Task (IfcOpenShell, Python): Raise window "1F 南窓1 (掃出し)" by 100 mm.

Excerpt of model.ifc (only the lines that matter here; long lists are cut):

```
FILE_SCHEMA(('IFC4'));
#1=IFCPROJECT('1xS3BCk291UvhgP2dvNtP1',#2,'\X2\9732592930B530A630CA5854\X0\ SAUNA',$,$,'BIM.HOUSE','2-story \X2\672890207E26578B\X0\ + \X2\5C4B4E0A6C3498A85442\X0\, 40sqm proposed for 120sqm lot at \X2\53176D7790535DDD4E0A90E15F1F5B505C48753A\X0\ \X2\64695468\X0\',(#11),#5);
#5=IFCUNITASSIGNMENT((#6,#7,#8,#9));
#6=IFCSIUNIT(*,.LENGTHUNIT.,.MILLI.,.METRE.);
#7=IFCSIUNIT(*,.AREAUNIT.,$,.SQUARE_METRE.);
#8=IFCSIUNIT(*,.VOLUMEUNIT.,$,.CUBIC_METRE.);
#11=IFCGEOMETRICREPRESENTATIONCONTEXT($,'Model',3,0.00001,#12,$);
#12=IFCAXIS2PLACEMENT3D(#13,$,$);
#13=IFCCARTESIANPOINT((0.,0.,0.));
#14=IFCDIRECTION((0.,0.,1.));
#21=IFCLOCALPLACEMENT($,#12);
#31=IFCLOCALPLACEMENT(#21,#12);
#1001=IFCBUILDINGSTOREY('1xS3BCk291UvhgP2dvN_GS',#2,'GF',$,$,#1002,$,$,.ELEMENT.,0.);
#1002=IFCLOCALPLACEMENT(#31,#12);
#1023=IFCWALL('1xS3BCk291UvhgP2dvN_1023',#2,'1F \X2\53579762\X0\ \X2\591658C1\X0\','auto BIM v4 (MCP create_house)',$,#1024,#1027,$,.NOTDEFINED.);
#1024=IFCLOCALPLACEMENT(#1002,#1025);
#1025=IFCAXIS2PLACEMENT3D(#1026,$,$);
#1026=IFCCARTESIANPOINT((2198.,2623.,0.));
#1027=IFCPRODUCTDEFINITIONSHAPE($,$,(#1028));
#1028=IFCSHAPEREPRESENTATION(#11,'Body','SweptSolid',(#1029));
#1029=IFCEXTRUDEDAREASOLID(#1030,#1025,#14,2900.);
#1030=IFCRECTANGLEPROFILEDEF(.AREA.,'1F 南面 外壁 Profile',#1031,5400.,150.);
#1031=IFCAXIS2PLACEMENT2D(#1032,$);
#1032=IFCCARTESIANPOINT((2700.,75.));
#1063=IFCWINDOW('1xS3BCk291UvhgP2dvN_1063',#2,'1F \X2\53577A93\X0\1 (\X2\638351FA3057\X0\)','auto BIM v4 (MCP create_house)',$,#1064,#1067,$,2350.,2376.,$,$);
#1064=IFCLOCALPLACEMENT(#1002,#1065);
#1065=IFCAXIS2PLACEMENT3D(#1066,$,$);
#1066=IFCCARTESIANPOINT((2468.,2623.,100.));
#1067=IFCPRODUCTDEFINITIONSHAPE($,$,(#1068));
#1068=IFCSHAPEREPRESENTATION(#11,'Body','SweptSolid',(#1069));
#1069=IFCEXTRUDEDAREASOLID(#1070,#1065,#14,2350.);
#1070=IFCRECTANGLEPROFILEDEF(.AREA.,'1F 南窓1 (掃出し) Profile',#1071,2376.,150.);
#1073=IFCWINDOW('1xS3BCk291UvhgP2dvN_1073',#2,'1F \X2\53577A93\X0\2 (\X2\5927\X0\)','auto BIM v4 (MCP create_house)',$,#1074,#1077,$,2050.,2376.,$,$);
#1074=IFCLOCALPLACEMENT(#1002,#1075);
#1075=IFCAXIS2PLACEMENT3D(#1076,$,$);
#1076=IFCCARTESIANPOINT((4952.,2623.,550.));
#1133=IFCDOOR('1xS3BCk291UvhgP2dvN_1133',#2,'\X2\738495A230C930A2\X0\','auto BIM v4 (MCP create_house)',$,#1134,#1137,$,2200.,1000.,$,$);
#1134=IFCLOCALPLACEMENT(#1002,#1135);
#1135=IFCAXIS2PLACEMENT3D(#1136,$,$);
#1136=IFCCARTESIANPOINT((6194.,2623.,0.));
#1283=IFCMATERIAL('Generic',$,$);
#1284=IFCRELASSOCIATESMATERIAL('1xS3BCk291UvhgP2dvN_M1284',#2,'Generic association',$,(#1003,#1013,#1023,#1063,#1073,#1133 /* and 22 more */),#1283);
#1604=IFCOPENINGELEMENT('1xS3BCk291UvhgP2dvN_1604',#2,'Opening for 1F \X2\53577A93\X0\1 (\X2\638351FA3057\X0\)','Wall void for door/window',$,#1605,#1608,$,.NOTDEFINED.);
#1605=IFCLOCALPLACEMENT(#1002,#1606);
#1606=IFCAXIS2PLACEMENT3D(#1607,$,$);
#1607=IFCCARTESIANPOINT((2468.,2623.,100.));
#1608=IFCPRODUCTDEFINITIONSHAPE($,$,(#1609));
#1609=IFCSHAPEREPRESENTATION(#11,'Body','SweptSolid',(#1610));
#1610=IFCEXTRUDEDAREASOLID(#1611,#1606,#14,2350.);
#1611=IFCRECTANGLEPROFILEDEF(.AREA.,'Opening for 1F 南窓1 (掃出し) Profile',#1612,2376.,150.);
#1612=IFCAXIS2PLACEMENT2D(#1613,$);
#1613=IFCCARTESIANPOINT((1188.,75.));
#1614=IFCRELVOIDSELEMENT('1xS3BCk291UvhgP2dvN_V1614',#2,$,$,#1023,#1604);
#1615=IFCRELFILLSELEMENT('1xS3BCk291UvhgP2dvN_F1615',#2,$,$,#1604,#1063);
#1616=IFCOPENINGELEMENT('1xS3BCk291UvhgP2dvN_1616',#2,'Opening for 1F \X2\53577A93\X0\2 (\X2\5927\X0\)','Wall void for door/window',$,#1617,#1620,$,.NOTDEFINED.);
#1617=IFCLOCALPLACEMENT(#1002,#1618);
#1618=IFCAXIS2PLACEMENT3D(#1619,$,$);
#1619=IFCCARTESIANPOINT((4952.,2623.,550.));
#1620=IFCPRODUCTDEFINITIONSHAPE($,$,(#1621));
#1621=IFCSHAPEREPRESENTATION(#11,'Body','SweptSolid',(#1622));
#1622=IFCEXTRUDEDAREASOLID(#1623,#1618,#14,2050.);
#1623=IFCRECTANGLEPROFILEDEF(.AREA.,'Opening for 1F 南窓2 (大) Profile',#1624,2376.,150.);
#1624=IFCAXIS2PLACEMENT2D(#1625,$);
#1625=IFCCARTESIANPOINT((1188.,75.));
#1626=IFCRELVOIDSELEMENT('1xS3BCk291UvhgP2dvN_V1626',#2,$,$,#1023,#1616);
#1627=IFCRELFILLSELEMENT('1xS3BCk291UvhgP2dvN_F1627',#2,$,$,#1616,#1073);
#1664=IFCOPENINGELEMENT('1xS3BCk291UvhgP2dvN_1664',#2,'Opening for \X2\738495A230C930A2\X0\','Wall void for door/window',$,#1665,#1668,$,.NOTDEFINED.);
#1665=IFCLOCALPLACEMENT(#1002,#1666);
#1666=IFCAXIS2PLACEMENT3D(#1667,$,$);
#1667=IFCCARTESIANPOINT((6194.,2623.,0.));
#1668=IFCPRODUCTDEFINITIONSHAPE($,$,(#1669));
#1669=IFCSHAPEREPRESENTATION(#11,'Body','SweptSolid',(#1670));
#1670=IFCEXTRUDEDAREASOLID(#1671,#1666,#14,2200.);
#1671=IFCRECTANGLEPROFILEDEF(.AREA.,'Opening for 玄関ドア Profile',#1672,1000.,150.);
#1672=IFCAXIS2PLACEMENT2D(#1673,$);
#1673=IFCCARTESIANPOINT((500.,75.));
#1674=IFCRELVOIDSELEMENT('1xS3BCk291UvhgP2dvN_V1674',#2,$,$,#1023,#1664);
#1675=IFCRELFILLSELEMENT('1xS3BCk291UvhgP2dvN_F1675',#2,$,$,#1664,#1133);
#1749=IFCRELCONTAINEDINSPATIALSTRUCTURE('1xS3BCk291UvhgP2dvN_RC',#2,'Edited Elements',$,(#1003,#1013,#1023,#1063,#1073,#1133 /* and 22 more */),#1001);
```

```python
import numpy as np
import ifcopenshell
import ifcopenshell.api.geometry
import ifcopenshell.util.placement
import ifcopenshell.util.unit

model = ifcopenshell.open("model.ifc")
unit_scale = ifcopenshell.util.unit.calculate_unit_scale(model)

window = model.by_guid("1xS3BCk291UvhgP2dvN_1063")
opening = window.FillsVoids[0].RelatingOpeningElement
dz = 0.1 / unit_scale

shift = np.array([0.0, 0.0, dz])
# The window is not placed relative to its opening, so move both.
for product in (opening, window):
    matrix = ifcopenshell.util.placement.get_local_placement(product.ObjectPlacement)
    matrix[:3, 3] += shift
    ifcopenshell.api.geometry.edit_object_placement(model, product=product, matrix=matrix, is_si=False)

print(f"moved by {dz * unit_scale:+.3f} m")

model.write("model_edited.ifc")
```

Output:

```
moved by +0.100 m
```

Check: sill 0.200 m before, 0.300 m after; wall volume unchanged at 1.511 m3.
